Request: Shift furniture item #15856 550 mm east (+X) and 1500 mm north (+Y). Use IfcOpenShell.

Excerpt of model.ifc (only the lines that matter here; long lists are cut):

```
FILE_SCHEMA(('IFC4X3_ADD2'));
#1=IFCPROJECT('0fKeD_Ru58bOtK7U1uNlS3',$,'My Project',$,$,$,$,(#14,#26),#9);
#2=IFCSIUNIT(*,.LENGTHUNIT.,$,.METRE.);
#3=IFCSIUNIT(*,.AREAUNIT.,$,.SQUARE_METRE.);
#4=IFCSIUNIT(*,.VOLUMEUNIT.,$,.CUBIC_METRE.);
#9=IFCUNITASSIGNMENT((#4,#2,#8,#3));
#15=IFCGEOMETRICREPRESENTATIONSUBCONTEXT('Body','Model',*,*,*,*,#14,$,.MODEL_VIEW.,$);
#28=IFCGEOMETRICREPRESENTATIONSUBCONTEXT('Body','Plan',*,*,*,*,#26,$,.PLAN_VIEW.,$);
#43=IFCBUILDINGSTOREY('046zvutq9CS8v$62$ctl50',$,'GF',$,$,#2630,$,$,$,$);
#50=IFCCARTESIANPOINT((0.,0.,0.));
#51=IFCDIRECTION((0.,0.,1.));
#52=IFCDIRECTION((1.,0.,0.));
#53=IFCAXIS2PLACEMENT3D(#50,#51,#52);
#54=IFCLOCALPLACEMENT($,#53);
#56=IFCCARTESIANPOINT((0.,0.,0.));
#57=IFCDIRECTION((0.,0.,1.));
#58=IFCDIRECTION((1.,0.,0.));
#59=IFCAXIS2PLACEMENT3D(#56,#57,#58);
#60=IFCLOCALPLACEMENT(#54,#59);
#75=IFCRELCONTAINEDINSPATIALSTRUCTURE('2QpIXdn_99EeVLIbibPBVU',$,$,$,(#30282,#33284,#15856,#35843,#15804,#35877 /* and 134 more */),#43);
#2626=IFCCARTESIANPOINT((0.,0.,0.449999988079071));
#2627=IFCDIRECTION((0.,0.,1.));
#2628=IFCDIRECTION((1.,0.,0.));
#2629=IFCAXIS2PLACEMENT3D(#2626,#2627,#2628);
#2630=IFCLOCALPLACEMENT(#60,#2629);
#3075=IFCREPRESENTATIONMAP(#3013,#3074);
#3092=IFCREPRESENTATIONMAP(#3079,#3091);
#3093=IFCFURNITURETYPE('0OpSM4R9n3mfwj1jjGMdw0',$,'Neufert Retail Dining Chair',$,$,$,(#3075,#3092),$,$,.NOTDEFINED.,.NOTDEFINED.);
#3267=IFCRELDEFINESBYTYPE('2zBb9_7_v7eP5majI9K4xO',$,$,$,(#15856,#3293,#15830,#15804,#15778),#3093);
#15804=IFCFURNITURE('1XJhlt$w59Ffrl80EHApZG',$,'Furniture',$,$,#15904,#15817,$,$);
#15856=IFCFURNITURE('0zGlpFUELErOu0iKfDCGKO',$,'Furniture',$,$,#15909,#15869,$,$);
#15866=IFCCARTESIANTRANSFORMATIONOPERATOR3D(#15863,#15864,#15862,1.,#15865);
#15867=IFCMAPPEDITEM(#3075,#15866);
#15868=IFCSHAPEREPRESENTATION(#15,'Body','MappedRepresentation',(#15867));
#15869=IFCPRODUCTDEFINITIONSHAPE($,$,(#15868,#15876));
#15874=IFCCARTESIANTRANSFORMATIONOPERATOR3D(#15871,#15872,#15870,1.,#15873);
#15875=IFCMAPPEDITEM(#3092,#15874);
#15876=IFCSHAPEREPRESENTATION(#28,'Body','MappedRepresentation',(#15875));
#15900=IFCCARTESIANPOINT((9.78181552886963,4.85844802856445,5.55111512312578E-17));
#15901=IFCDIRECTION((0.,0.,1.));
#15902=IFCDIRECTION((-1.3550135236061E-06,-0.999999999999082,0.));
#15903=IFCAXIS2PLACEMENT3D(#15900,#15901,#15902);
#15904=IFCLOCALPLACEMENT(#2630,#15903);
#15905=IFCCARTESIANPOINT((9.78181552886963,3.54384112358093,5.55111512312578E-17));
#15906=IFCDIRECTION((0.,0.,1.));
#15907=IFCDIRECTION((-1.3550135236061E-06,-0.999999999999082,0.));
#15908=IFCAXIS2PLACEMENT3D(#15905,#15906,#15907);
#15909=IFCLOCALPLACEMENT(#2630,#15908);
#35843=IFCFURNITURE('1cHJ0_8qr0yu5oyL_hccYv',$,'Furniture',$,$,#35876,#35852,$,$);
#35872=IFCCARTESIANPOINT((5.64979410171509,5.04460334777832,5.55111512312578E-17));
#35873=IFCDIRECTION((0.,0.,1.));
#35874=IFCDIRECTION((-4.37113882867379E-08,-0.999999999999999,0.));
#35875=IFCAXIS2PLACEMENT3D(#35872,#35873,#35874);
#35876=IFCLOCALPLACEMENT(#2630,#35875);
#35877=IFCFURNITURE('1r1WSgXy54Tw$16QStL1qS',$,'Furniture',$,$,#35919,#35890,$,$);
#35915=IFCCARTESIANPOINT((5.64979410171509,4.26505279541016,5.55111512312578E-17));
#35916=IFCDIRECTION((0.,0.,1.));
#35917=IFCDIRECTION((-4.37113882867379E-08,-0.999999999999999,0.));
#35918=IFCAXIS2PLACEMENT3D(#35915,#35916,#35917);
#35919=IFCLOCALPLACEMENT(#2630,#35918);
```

```python
import ifcopenshell
import ifcopenshell.api.geometry
import ifcopenshell.util.placement

model = ifcopenshell.open("model.ifc")

item = model.by_guid("0zGlpFUELErOu0iKfDCGKO")
matrix = ifcopenshell.util.placement.get_local_placement(item.ObjectPlacement)
matrix[0, 3] += 0.55
matrix[1, 3] += 1.5
ifcopenshell.api.geometry.edit_object_placement(model, product=item, matrix=matrix, is_si=False)

print(ifcopenshell.util.placement.get_local_placement(item.ObjectPlacement).round(3) + 0.0)

model.write("model_rev.ifc")
```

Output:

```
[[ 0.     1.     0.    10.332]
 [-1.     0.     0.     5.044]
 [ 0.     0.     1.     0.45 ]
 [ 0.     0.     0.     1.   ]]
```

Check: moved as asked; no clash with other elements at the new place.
